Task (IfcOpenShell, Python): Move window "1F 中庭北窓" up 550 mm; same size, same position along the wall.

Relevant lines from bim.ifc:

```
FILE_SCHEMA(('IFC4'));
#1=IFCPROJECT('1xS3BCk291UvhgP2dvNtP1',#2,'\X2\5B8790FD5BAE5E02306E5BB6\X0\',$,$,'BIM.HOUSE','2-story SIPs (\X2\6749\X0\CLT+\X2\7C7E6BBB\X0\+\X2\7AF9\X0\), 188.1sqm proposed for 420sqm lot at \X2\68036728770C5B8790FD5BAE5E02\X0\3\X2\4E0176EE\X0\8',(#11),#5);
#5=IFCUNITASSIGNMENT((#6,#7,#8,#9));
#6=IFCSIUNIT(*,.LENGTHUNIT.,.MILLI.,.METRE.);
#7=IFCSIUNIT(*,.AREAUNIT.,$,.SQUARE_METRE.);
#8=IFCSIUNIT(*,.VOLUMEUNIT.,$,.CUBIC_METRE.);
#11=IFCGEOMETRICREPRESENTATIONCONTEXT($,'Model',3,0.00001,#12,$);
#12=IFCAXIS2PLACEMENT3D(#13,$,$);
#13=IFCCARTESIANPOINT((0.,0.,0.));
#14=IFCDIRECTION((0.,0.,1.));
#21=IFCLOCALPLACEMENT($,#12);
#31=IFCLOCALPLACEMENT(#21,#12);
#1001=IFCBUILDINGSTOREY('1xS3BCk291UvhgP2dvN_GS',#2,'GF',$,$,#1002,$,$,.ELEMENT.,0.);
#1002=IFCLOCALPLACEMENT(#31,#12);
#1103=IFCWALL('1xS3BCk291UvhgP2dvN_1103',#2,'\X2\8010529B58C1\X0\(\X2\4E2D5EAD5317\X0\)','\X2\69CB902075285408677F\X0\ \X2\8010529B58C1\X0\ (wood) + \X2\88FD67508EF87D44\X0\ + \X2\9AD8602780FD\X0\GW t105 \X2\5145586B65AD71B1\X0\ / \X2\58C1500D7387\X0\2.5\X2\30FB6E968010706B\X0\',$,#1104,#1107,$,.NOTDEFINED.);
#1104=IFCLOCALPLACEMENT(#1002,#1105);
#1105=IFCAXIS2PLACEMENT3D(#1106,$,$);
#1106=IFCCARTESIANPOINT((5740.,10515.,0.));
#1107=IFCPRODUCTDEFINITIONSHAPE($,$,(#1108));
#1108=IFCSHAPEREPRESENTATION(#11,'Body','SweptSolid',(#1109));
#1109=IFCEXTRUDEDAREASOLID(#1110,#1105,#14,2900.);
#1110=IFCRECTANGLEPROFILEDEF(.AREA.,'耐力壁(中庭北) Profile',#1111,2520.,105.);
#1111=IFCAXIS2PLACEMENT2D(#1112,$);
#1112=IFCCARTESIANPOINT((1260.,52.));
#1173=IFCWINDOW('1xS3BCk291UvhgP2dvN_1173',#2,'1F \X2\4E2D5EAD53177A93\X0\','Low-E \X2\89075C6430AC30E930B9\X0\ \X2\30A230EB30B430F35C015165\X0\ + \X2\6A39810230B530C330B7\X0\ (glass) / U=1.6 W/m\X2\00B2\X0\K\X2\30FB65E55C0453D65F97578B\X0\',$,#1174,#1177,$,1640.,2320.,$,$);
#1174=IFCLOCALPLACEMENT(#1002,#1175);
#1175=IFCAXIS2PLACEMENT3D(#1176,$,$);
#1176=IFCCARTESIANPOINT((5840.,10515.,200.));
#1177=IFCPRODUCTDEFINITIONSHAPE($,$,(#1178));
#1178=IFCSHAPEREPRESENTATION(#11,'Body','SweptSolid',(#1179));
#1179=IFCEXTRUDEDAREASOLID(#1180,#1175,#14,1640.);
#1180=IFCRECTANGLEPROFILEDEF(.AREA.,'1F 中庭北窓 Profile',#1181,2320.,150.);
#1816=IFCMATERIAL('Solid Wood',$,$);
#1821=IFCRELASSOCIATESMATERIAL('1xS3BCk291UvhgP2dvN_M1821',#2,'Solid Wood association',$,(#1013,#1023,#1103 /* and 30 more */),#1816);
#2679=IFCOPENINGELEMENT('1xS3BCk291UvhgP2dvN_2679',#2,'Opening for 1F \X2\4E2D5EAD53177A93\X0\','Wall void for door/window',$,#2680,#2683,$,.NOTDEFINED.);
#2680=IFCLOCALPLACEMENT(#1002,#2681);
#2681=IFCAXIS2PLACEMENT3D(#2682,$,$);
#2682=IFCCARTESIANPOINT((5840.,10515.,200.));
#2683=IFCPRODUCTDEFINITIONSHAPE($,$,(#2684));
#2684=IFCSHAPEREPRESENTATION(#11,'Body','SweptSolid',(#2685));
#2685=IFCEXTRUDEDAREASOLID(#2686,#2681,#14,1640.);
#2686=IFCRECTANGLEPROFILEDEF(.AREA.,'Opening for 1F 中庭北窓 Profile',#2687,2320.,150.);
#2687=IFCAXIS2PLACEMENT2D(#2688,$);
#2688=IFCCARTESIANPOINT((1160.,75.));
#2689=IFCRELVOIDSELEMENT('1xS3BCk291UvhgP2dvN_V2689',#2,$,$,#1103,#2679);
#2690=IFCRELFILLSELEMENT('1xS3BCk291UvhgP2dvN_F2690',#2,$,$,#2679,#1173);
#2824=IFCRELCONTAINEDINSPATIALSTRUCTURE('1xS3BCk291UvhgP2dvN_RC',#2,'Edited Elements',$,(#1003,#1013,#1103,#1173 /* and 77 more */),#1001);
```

```python
import numpy as np
import ifcopenshell
import ifcopenshell.api.geometry
import ifcopenshell.util.placement
import ifcopenshell.util.unit

model = ifcopenshell.open("bim.ifc")
unit_scale = ifcopenshell.util.unit.calculate_unit_scale(model)

window = model.by_guid("1xS3BCk291UvhgP2dvN_1173")
opening = window.FillsVoids[0].RelatingOpeningElement
dz = 0.55 / unit_scale

shift = np.array([0.0, 0.0, dz])
# The window is not placed relative to its opening, so move both.
for product in (opening, window):
    matrix = ifcopenshell.util.placement.get_local_placement(product.ObjectPlacement)
    matrix[:3, 3] += shift
    ifcopenshell.api.geometry.edit_object_placement(model, product=product, matrix=matrix, is_si=False)

print(f"moved by {dz * unit_scale:+.3f} m")

model.write("bim_edited.ifc")
```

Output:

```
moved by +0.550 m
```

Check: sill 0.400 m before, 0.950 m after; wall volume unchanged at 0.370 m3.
